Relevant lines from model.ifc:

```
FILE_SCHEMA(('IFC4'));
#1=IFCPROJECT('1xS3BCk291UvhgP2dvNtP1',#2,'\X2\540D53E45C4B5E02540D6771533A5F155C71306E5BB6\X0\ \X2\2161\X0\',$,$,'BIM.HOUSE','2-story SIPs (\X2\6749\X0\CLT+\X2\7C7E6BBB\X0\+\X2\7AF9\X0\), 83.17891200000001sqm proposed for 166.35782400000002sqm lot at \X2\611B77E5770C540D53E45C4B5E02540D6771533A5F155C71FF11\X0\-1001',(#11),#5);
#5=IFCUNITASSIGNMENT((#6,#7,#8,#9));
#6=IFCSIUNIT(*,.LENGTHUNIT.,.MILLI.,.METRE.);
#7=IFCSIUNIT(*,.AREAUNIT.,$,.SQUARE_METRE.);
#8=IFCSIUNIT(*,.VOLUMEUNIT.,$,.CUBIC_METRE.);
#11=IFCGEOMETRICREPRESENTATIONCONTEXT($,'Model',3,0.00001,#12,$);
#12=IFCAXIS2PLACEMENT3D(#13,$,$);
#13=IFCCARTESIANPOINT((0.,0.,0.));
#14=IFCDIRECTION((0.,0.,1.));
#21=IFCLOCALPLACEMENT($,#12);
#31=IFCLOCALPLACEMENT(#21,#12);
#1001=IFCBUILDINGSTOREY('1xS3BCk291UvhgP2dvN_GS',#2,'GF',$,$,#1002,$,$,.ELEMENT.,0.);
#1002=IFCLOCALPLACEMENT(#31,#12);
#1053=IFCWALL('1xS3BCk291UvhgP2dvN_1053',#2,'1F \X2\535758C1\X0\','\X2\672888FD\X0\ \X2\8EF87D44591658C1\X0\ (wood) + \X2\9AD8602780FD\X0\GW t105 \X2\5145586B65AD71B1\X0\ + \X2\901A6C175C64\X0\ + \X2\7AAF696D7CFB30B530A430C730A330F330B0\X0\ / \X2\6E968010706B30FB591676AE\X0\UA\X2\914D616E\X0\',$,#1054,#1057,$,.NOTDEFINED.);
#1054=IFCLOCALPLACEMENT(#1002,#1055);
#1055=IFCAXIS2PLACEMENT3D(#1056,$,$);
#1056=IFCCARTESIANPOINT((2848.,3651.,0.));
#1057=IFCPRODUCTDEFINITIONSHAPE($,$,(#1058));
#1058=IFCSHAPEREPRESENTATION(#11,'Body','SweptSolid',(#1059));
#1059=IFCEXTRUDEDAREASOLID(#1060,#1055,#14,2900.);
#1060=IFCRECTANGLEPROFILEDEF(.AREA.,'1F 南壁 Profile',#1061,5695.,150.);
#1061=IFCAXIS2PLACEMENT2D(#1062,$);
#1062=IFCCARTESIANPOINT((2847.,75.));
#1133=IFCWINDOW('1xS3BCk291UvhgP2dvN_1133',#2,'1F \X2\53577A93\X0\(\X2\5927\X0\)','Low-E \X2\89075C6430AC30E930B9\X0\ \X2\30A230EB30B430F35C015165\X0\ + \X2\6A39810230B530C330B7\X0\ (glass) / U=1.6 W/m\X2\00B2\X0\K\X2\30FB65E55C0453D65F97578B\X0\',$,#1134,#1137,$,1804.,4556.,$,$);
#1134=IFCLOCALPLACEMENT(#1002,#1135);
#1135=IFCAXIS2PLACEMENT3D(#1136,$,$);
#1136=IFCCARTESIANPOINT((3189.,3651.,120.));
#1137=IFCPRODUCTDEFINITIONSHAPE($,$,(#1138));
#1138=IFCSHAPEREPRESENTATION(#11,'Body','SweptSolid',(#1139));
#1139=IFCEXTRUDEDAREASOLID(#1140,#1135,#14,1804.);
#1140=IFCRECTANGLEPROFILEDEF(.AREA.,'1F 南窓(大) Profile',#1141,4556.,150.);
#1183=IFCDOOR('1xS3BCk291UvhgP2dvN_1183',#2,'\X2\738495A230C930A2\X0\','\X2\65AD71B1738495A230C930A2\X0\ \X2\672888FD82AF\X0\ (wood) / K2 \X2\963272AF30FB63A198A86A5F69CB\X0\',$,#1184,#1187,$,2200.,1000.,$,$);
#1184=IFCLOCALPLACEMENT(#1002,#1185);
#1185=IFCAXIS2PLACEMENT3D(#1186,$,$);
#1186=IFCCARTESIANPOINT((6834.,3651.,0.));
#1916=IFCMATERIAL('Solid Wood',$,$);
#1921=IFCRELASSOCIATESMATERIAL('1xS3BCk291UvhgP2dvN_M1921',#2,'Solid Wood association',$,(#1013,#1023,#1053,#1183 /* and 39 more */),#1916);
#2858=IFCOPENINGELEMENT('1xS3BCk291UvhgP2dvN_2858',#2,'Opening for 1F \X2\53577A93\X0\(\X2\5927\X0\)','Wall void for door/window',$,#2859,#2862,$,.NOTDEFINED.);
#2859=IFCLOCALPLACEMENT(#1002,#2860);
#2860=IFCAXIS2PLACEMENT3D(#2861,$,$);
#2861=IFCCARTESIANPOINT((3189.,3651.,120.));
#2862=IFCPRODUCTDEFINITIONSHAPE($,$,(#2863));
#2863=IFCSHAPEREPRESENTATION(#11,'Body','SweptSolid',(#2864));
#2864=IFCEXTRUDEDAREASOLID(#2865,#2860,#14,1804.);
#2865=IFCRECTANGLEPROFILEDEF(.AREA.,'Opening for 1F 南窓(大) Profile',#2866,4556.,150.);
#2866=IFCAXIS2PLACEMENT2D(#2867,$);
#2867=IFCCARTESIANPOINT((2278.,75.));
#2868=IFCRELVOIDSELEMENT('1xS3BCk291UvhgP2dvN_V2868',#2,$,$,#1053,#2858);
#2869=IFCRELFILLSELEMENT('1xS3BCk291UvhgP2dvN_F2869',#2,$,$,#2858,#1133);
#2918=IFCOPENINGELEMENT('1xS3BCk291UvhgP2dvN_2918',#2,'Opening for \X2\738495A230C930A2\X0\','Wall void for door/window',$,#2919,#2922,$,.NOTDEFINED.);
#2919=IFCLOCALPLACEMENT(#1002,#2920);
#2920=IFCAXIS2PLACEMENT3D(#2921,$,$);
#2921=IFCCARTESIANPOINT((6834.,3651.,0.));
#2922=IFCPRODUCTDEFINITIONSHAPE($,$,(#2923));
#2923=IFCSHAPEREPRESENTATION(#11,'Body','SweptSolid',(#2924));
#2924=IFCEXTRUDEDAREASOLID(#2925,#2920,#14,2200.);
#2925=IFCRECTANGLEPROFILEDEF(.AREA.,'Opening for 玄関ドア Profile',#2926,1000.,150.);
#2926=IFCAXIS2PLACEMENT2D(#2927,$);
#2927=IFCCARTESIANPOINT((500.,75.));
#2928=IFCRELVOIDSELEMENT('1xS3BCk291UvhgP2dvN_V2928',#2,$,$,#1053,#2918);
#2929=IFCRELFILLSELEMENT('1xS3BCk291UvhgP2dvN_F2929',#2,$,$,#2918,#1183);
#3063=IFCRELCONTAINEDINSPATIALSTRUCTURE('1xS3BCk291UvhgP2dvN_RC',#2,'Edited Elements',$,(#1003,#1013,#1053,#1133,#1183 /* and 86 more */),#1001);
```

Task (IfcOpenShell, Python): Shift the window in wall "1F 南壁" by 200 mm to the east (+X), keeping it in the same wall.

```python
import ifcopenshell
import ifcopenshell.api.geometry
import ifcopenshell.util.placement
import ifcopenshell.util.unit

model = ifcopenshell.open("model.ifc")
unit_scale = ifcopenshell.util.unit.calculate_unit_scale(model)

window = model.by_id(1133)
opening = window.FillsVoids[0].RelatingOpeningElement
wall = opening.VoidsElements[0].RelatingBuildingElement

wall_matrix = ifcopenshell.util.placement.get_local_placement(wall.ObjectPlacement)
shift = wall_matrix[:3, 0] * 0.2 / unit_scale
before = ifcopenshell.util.placement.get_local_placement(window.ObjectPlacement)[:3, 3].copy()

# The window is not placed relative to its opening, so move both.
for product in (opening, window):
    matrix = ifcopenshell.util.placement.get_local_placement(product.ObjectPlacement)
    matrix[:3, 3] += shift
    ifcopenshell.api.geometry.edit_object_placement(model, product=product, matrix=matrix, is_si=False)

after = ifcopenshell.util.placement.get_local_placement(window.ObjectPlacement)[:3, 3]
print("window moved by", (after - before).round(3) + 0.0)

model.write("model_rev.ifc")
```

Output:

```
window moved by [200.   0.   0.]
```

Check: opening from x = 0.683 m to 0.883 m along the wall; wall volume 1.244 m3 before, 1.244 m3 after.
